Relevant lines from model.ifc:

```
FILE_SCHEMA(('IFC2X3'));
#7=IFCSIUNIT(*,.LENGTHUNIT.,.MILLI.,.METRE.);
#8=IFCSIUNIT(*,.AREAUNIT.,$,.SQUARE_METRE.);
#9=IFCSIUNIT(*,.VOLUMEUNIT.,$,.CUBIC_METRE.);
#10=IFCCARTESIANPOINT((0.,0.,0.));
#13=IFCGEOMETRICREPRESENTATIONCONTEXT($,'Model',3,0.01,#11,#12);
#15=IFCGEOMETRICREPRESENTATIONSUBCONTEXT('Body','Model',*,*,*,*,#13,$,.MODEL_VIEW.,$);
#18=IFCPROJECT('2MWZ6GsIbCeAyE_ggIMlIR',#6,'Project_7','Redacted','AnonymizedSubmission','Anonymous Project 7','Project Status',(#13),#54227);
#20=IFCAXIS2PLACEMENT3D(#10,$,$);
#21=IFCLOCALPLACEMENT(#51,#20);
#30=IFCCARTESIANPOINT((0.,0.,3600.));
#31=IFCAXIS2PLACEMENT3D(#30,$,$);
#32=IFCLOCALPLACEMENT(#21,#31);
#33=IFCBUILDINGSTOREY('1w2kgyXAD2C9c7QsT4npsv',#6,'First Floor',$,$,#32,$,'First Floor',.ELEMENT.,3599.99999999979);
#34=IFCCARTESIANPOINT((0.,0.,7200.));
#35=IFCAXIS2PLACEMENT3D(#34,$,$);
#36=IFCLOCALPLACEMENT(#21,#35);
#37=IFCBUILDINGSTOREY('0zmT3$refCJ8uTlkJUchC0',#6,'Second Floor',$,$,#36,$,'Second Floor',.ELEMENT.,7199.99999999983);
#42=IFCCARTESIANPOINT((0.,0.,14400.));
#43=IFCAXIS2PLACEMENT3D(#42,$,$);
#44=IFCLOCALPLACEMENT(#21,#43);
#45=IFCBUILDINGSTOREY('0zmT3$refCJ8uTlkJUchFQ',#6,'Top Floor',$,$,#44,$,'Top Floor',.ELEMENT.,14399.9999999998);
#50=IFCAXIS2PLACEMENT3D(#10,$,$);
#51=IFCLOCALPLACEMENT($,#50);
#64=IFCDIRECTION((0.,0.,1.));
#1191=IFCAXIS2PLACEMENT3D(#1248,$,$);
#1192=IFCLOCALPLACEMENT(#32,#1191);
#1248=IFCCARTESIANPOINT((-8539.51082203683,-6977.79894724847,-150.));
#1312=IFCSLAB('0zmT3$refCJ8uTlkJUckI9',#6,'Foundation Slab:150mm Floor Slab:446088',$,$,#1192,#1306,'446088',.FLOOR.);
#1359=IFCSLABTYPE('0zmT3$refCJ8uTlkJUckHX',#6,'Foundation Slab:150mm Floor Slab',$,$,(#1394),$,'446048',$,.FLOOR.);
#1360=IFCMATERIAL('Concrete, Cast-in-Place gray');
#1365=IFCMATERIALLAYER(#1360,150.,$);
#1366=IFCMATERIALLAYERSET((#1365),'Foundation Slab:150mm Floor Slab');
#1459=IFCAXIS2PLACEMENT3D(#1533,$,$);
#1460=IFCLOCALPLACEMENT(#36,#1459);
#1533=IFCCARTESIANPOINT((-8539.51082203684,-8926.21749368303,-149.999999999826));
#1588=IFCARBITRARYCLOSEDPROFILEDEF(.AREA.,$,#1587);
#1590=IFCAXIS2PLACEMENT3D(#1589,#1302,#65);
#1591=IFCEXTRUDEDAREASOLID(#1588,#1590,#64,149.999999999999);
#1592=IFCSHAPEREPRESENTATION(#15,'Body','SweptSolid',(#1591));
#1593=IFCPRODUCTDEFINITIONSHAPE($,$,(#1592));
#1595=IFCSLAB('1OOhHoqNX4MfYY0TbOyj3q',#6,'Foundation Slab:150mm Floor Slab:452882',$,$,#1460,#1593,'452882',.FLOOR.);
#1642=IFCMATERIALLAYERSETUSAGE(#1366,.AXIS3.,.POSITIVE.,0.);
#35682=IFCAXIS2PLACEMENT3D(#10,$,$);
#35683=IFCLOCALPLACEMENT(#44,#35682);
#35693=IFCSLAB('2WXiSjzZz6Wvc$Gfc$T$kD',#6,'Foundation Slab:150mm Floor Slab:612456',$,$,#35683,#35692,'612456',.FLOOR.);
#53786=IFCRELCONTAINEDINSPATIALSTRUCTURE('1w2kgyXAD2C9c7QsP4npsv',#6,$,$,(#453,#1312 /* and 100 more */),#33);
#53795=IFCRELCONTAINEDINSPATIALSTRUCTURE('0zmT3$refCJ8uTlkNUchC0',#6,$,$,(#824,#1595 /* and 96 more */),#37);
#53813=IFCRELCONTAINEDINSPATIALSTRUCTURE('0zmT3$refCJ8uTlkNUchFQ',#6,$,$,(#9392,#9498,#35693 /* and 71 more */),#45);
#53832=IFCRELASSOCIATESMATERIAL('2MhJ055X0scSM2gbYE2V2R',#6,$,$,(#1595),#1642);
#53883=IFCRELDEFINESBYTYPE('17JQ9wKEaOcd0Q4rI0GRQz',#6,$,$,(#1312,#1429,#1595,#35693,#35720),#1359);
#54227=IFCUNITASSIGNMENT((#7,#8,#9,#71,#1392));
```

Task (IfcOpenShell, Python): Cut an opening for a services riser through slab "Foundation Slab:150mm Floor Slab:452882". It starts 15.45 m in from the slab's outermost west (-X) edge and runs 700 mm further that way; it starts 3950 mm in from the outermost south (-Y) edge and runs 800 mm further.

```python
import numpy as np
import ifcopenshell
import ifcopenshell.api.feature
import ifcopenshell.api.geometry
import ifcopenshell.api.root
import ifcopenshell.geom
import ifcopenshell.util.placement
import ifcopenshell.util.representation
import ifcopenshell.util.shape
import ifcopenshell.util.unit

model = ifcopenshell.open("model.ifc")
unit_scale = ifcopenshell.util.unit.calculate_unit_scale(model)
settings = ifcopenshell.geom.settings()


def volume(element):
    """Net volume in cubic metres, openings subtracted."""
    shape = ifcopenshell.geom.create_shape(settings, element)
    return ifcopenshell.util.shape.get_volume(shape.geometry)


slab = model.by_guid("1OOhHoqNX4MfYY0TbOyj3q")
before = volume(slab)

# Extent in the slab's own axes, in metres. The edges named are its -X and -Y sides.
slab_shape = ifcopenshell.geom.create_shape(settings, slab)
vertices = ifcopenshell.util.shape.get_vertices(slab_shape.geometry)
x_min, y_min, bottom = vertices.min(axis=0)
top = vertices[:, 2].max()

opening = ifcopenshell.api.root.create_entity(model, ifc_class="IfcOpeningElement", name="Services riser opening")
context = ifcopenshell.util.representation.get_context(model, "Model", "Body", "MODEL_VIEW")
width, depth = 0.7, 0.8
outline = [(0.0, 0.0), (width, 0.0), (width, depth), (0.0, depth), (0.0, 0.0)]
# Overshoot both faces by 50 mm so the cut is clean.
shape = ifcopenshell.api.geometry.add_slab_representation(
    model, context=context, depth=top - bottom + 0.1, polyline=outline
)
ifcopenshell.api.geometry.assign_representation(model, product=opening, representation=shape)

matrix = ifcopenshell.util.placement.get_local_placement(slab.ObjectPlacement)
matrix[:, 3] = matrix @ np.append(np.array([x_min + 15.45, y_min + 3.95, bottom - 0.05]) / unit_scale, 1.0)
ifcopenshell.api.geometry.edit_object_placement(model, product=opening, matrix=matrix, is_si=False)
ifcopenshell.api.feature.add_feature(model, feature=opening, element=slab)

after = volume(slab)

print(f"slab volume {before:.3f} -> {after:.3f} m3")

model.write("model-out.ifc")
```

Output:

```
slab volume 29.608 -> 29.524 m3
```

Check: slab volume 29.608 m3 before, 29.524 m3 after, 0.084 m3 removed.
